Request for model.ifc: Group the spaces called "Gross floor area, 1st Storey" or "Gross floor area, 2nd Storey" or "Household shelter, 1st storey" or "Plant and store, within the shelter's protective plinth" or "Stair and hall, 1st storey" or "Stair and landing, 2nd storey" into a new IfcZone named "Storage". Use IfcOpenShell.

First a look at what the model holds.

```python
import ifcopenshell

model = ifcopenshell.open("model.ifc")
print(model.schema)
seen = {}
for space in model.by_type("IfcSpace"):
    seen[space.LongName] = seen.get(space.LongName, 0) + 1
for name, count in sorted(seen.items(), key=str):
    print(count, "x", name)
print("zones:", [z.Name for z in model.by_type("IfcZone")][:20])
```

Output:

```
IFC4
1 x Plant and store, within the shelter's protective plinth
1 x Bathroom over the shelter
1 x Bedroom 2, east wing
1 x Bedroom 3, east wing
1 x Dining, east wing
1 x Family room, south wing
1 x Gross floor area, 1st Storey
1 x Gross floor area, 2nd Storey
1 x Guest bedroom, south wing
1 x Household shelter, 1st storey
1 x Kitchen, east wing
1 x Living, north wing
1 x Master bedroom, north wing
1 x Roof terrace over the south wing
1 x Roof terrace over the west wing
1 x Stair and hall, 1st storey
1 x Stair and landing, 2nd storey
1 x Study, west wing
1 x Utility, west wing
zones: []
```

```python
import ifcopenshell
import ifcopenshell.api.group
import ifcopenshell.api.root

model = ifcopenshell.open("model.ifc")

names = {"Gross floor area, 1st Storey", "Gross floor area, 2nd Storey", "Household shelter, 1st storey", "Plant and store, within the shelter's protective plinth", "Stair and hall, 1st storey", "Stair and landing, 2nd storey"}
spaces = [s for s in model.by_type("IfcSpace") if s.LongName in names]

zone = ifcopenshell.api.root.create_entity(model, ifc_class="IfcZone", name="Storage")
ifcopenshell.api.group.assign_group(model, products=spaces, group=zone)
print(len(spaces), "spaces in", zone.Name)

model.write("model-out.ifc")
```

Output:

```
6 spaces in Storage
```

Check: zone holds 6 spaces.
